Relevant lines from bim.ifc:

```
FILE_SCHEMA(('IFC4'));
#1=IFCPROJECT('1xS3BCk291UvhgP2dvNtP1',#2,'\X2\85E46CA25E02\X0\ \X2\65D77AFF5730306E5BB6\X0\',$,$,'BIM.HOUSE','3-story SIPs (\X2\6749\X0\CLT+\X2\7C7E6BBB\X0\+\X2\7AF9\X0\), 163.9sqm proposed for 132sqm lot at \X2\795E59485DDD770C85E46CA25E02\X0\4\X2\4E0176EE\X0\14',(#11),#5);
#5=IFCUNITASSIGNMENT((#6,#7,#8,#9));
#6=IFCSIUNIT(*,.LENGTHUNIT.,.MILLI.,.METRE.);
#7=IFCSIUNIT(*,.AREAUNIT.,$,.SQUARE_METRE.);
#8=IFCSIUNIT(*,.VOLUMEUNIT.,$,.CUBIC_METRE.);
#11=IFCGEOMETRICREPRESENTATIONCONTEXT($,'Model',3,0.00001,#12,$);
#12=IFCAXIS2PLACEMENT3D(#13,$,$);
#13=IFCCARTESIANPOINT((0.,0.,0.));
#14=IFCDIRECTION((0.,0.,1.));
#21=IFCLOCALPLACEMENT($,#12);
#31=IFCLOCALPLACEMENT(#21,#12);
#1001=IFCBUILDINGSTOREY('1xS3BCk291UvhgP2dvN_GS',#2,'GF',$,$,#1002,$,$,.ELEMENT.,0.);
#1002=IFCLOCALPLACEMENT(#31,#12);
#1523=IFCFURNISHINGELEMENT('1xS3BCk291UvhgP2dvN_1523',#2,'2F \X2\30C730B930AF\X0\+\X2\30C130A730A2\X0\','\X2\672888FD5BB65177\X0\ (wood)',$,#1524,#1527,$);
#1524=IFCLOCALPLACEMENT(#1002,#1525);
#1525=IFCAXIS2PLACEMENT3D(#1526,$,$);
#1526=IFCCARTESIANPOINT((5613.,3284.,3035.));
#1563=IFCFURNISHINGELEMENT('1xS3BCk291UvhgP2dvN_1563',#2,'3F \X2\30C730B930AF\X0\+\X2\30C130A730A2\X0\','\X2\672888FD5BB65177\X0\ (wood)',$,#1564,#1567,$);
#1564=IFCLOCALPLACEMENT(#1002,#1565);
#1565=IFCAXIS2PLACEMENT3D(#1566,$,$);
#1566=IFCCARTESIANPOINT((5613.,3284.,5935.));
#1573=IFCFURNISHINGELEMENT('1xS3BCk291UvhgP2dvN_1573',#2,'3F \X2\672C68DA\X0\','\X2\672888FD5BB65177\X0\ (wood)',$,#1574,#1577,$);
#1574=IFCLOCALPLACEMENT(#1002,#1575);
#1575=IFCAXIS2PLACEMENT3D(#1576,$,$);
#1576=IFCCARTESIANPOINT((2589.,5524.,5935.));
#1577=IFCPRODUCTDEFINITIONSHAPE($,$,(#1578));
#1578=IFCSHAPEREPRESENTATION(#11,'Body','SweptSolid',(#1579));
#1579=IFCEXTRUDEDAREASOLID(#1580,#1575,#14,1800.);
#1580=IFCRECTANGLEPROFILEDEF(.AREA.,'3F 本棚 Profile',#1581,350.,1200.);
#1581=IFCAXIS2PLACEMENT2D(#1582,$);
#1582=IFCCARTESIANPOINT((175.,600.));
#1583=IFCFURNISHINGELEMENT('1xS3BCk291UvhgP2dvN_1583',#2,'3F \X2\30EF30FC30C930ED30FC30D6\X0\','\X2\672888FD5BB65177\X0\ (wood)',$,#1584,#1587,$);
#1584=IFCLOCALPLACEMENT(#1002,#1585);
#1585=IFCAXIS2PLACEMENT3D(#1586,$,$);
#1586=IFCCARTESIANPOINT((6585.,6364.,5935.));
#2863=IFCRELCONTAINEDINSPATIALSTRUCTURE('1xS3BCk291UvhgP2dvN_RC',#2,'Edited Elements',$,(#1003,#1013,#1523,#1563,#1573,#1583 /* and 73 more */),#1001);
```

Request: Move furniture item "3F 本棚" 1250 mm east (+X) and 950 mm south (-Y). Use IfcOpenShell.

```python
import ifcopenshell
import ifcopenshell.api.geometry
import ifcopenshell.util.placement

model = ifcopenshell.open("bim.ifc")

item = model.by_guid("1xS3BCk291UvhgP2dvN_1573")
matrix = ifcopenshell.util.placement.get_local_placement(item.ObjectPlacement)
matrix[0, 3] += 1250.0
matrix[1, 3] -= 950.0
ifcopenshell.api.geometry.edit_object_placement(model, product=item, matrix=matrix, is_si=False)

print(ifcopenshell.util.placement.get_local_placement(item.ObjectPlacement).round(3) + 0.0)

model.write("bim_v2.ifc")
```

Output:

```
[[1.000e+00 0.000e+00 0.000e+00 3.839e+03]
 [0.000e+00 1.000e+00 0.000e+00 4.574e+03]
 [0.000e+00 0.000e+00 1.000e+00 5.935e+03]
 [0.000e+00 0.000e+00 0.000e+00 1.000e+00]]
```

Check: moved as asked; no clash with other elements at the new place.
